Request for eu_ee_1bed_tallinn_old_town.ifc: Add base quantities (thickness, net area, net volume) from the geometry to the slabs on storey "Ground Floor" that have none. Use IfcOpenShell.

First a look at what the model holds.

```python
import ifcopenshell
import ifcopenshell.util.element
import ifcopenshell.util.unit

model = ifcopenshell.open("eu_ee_1bed_tallinn_old_town.ifc")
print(model.schema)
for unit_type in ("LENGTHUNIT", "AREAUNIT", "VOLUMEUNIT"):
    print(unit_type, ifcopenshell.util.unit.calculate_unit_scale(model, unit_type))
storey = next(s for s in model.by_type("IfcBuildingStorey") if s.Name == "Ground Floor")
slabs = [e for e in ifcopenshell.util.element.get_decomposition(storey) if e.is_a("IfcSlab")]
for e in sorted(slabs, key=lambda e: e.id()):
    print(e.id(), e.is_a(), e.Name, list(ifcopenshell.util.element.get_psets(e, qtos_only=True)), sep=" | ")
```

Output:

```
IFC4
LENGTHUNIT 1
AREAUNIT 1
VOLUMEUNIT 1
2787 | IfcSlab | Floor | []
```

```python
import ifcopenshell
import ifcopenshell.api.pset
import ifcopenshell.geom
import ifcopenshell.util.element
import ifcopenshell.util.shape
import ifcopenshell.util.unit

model = ifcopenshell.open("eu_ee_1bed_tallinn_old_town.ifc")
unit_scale = ifcopenshell.util.unit.calculate_unit_scale(model)
area_scale = ifcopenshell.util.unit.calculate_unit_scale(model, "AREAUNIT")
volume_scale = ifcopenshell.util.unit.calculate_unit_scale(model, "VOLUMEUNIT")
settings = ifcopenshell.geom.settings()

storey = next(s for s in model.by_type("IfcBuildingStorey") if s.Name == "Ground Floor")
slabs = [e for e in ifcopenshell.util.element.get_decomposition(storey) if e.is_a("IfcSlab")]

for e in sorted(slabs, key=lambda e: e.id()):
    if ifcopenshell.util.element.get_psets(e, qtos_only=True, should_inherit=False):
        continue
    # Geometry comes back in metres, in the element's own axes.
    shape = ifcopenshell.geom.create_shape(settings, e)
    values = {
        "Width": ifcopenshell.util.shape.get_z(shape.geometry) / unit_scale,
        "NetArea": ifcopenshell.util.shape.get_footprint_area(shape.geometry) / area_scale,
        "NetVolume": ifcopenshell.util.shape.get_volume(shape.geometry) / volume_scale,
    }
    qto = ifcopenshell.api.pset.add_qto(model, product=e, name="Qto_SlabBaseQuantities")
    ifcopenshell.api.pset.edit_qto(model, qto=qto, properties=values)
    print(e.id(), {k: round(v, 3) for k, v in values.items()})

model.write("eu_ee_1bed_tallinn_old_town_updated.ifc")
```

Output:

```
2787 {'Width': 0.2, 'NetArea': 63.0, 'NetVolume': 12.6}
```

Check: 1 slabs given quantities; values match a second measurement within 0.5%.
